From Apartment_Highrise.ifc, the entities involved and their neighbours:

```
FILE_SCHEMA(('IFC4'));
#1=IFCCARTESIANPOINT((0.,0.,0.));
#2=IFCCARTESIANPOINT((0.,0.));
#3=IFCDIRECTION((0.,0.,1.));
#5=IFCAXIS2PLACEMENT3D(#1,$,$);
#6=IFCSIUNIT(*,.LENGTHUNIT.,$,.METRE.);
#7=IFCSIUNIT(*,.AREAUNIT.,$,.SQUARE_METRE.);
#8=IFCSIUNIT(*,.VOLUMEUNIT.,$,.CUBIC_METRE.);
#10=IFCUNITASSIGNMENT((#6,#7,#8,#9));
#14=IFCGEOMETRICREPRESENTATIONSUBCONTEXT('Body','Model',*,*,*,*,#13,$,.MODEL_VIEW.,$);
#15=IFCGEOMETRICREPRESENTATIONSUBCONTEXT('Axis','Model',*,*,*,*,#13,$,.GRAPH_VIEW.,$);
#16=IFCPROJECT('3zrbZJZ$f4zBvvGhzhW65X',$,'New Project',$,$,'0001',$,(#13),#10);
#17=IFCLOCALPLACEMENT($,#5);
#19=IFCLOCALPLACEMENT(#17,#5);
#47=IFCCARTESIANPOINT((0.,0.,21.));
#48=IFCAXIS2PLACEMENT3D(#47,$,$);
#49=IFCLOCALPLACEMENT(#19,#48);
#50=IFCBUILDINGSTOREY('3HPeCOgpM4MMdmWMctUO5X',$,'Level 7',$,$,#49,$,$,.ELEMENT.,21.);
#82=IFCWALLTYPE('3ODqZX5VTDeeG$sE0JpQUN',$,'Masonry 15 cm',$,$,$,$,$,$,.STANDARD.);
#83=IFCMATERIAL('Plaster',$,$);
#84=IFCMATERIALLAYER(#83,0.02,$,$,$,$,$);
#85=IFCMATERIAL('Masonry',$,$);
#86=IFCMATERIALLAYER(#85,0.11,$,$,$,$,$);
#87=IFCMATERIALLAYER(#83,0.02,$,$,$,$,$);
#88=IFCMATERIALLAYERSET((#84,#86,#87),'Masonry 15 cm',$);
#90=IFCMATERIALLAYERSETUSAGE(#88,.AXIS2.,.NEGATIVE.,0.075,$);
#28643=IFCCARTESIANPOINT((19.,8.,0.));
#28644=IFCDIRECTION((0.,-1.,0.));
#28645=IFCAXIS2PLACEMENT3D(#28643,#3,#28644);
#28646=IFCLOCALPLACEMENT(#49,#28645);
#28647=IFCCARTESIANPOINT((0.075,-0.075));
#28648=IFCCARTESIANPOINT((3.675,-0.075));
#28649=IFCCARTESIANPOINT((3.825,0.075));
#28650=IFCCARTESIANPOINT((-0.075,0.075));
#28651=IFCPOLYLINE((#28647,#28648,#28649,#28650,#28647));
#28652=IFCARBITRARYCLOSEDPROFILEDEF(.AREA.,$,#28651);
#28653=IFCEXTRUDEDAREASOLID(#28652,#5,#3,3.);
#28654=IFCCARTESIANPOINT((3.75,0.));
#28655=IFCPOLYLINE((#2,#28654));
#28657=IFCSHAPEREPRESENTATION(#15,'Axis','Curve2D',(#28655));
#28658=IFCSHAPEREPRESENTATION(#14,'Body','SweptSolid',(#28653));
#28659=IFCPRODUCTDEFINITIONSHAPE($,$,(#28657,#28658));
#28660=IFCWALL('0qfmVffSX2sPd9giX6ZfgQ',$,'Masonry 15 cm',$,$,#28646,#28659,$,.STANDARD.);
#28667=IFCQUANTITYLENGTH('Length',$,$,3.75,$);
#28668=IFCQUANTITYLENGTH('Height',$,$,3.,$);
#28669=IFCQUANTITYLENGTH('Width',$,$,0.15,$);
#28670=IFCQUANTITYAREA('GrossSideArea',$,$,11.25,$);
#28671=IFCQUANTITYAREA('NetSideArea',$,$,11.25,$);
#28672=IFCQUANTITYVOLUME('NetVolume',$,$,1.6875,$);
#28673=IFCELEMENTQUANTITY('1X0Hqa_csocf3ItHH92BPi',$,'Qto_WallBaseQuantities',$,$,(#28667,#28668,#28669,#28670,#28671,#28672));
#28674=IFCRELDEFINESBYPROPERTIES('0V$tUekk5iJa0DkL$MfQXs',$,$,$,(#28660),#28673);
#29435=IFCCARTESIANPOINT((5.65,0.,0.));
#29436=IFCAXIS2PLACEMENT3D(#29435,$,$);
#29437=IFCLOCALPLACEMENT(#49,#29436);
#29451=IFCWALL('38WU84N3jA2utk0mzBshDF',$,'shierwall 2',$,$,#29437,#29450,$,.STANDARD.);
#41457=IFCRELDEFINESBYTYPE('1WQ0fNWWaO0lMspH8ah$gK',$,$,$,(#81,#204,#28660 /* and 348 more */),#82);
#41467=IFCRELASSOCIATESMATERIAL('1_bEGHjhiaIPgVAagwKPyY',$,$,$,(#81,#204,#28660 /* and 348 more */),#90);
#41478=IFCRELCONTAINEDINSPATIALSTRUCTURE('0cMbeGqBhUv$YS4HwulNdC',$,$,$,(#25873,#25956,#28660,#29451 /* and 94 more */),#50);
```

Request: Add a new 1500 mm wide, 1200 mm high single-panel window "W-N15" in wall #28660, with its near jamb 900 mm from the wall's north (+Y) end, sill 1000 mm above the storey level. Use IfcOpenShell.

```python
import numpy as np
import ifcopenshell
import ifcopenshell.api.feature
import ifcopenshell.api.geometry
import ifcopenshell.api.pset
import ifcopenshell.api.root
import ifcopenshell.api.spatial
import ifcopenshell.geom
import ifcopenshell.util.element
import ifcopenshell.util.placement
import ifcopenshell.util.representation
import ifcopenshell.util.shape
import ifcopenshell.util.unit

model = ifcopenshell.open("Apartment_Highrise.ifc")
unit_scale = ifcopenshell.util.unit.calculate_unit_scale(model)
area_scale = ifcopenshell.util.unit.calculate_unit_scale(model, "AREAUNIT")
volume_scale = ifcopenshell.util.unit.calculate_unit_scale(model, "VOLUMEUNIT")
settings = ifcopenshell.geom.settings()


def volume(element):
    """Net volume in cubic metres, openings subtracted."""
    shape = ifcopenshell.geom.create_shape(settings, element)
    return ifcopenshell.util.shape.get_volume(shape.geometry)


wall = model.by_id(28660)
storey = ifcopenshell.util.element.get_container(wall, ifc_class="IfcBuildingStorey")
context = ifcopenshell.util.representation.get_context(model, "Model", "Body", "MODEL_VIEW")
before = volume(wall)

width, height, from_end, sill = 1.5, 1.2, 0.9, 1  # metres

# The wall runs along its own X axis, and the end named is its -X end.
wall_shape = ifcopenshell.geom.create_shape(settings, wall)
x, y, z = ifcopenshell.util.shape.get_vertices(wall_shape.geometry).T
start = x.min() + from_end
face, thickness = float(y.min()), float(y.max() - y.min())
wall_matrix = ifcopenshell.util.placement.get_local_placement(wall.ObjectPlacement)
level = ifcopenshell.util.placement.get_local_placement(storey.ObjectPlacement)[2, 3]


def in_wall(x, y):
    """Placement at x, y metres in the wall's axes, at sill height."""
    matrix = wall_matrix.copy()
    matrix[:, 3] = wall_matrix @ np.array([x / unit_scale, y / unit_scale, 0.0, 1.0])
    matrix[2, 3] = level + sill / unit_scale
    return matrix


# Opening: a box that overshoots both wall faces by 50 mm.
opening = ifcopenshell.api.root.create_entity(model, ifc_class="IfcOpeningElement", predefined_type="OPENING")
box = ifcopenshell.api.geometry.add_wall_representation(
    model, context=context, length=width, height=height, thickness=thickness + 0.1
)
ifcopenshell.api.geometry.assign_representation(model, product=opening, representation=box)
ifcopenshell.api.geometry.edit_object_placement(model, product=opening, matrix=in_wall(start, face - 0.05), is_si=False)
ifcopenshell.api.feature.add_feature(model, feature=opening, element=wall)

window = ifcopenshell.api.root.create_entity(model, ifc_class="IfcWindow", name="W-N15", predefined_type="WINDOW")
window.OverallWidth, window.OverallHeight = width / unit_scale, height / unit_scale
window.PartitioningType = "SINGLE_PANEL"
body = ifcopenshell.api.geometry.add_window_representation(
    model,
    context=context,
    overall_width=window.OverallWidth,
    overall_height=window.OverallHeight,
    partition_type="SINGLE_PANEL",
)
ifcopenshell.api.geometry.assign_representation(model, product=window, representation=body)
ifcopenshell.api.spatial.assign_container(model, products=[window], relating_structure=storey)
ifcopenshell.api.feature.add_filling(model, opening=opening, element=window)

# Centre the window in the wall's thickness.
ifcopenshell.api.geometry.edit_object_placement(model, product=window, matrix=in_wall(start, face), is_si=False)
window_shape = ifcopenshell.geom.create_shape(settings, window)
depth = ifcopenshell.util.shape.get_vertices(window_shape.geometry)[:, 1]
offset = face + thickness / 2 - (depth.min() + depth.max()) / 2
ifcopenshell.api.geometry.edit_object_placement(model, product=window, matrix=in_wall(start, offset), is_si=False)

after = volume(wall)

# Update the wall's stored quantities.
qto = model.by_id(ifcopenshell.util.element.get_pset(wall, "Qto_WallBaseQuantities", should_inherit=False)["id"])
ifcopenshell.api.pset.edit_qto(model, qto=qto, properties={
    "NetSideArea": after / thickness / area_scale,
    "NetVolume": after / volume_scale,
})

print(f"wall volume {before:.3f} -> {after:.3f} m3")

model.write("Apartment_Highrise_rev.ifc")
```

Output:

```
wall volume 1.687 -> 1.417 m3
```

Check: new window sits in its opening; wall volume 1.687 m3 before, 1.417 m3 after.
